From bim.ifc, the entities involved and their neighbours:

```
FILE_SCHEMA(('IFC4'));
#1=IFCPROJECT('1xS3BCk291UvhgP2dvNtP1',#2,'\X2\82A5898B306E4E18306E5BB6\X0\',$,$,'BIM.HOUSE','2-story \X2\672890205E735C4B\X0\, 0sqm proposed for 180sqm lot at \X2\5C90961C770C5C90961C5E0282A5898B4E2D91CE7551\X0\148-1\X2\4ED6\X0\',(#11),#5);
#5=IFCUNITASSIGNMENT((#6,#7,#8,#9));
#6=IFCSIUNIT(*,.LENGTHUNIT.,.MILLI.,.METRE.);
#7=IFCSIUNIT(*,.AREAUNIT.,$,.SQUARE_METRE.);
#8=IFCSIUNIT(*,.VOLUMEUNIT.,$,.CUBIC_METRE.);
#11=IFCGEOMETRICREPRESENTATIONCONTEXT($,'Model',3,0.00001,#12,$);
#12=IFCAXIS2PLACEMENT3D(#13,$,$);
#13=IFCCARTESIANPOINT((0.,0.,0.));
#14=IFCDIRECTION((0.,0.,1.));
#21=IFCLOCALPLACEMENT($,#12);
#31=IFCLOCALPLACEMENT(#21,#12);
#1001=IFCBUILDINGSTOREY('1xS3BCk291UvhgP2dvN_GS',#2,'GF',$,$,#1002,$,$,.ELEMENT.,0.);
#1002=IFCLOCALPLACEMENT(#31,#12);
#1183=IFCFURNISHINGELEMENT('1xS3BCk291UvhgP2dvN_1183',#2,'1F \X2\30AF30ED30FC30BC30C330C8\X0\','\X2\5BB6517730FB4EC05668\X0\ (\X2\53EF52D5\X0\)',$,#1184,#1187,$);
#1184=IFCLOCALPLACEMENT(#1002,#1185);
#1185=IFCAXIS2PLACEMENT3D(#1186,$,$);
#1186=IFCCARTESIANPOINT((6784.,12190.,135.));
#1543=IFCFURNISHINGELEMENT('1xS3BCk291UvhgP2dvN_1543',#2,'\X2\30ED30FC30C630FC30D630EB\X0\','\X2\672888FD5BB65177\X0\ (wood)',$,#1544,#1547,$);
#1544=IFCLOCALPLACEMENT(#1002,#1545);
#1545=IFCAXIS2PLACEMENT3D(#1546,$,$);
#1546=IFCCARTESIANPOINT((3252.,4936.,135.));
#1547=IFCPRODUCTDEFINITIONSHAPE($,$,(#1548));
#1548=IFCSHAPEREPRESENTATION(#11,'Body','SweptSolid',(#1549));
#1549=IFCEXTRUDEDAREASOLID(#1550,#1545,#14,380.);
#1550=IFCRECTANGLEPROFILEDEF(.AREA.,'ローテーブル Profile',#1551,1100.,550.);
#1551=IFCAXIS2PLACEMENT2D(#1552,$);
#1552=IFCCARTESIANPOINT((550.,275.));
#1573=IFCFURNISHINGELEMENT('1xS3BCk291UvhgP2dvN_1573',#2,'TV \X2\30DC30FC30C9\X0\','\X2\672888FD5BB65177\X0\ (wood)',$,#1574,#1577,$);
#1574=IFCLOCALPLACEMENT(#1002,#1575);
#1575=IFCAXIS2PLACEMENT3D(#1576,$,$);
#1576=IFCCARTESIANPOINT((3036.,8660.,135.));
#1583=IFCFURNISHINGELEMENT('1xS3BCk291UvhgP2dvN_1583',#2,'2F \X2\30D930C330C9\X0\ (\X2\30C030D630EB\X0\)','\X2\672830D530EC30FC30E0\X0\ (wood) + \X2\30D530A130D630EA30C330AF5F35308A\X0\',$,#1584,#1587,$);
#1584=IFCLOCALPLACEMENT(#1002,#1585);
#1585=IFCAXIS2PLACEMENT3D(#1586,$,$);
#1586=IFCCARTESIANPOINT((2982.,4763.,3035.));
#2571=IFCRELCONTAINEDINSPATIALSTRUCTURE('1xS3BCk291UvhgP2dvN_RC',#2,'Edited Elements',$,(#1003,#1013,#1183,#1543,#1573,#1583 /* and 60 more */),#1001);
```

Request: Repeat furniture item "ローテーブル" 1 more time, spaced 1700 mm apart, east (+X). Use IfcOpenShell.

```python
import numpy as np
import ifcopenshell
import ifcopenshell.api.geometry
import ifcopenshell.api.root
import ifcopenshell.util.element
import ifcopenshell.util.placement
import ifcopenshell.util.unit

model = ifcopenshell.open("bim.ifc")
unit_scale = ifcopenshell.util.unit.calculate_unit_scale(model)


def reuse_history(source, copy):
    """copy_class also copies each property set's owner history, people and application; keep the originals."""
    for rel in copy.IsDefinedBy:
        if rel.is_a("IfcRelDefinesByProperties") and (history := rel.RelatingPropertyDefinition.OwnerHistory):
            rel.RelatingPropertyDefinition.OwnerHistory = source.OwnerHistory
            ifcopenshell.util.element.remove_deep2(model, history)


source = model.by_id(1543)
base = ifcopenshell.util.placement.get_local_placement(source.ObjectPlacement)
step = np.array([1.0, 0.0, 0.0]) * 1.7 / unit_scale

for i in range(1, 2):
    copy = ifcopenshell.api.root.copy_class(model, product=source)
    copy.Representation = ifcopenshell.util.element.copy_deep(
        model, source.Representation, exclude=["IfcGeometricRepresentationContext", "IfcRepresentationMap"]
    )
    reuse_history(source, copy)
    matrix = base.copy()
    matrix[:3, 3] += i * step
    print("added at", matrix[:3, 3].round(3) + 0.0)
    ifcopenshell.api.geometry.edit_object_placement(model, product=copy, matrix=matrix, is_si=False)

model.write("bim-out.ifc")
```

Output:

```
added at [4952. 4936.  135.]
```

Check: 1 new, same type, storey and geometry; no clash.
